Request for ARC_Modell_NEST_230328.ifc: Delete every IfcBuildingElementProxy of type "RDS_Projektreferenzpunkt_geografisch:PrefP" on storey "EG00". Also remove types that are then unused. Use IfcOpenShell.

First a look at what the model holds.

```python
import ifcopenshell
import ifcopenshell.util.element

model = ifcopenshell.open("ARC_Modell_NEST_230328.ifc")
print(model.schema)
storey = next(s for s in model.by_type("IfcBuildingStorey") if s.Name == "EG00")
proxies = [e for e in ifcopenshell.util.element.get_decomposition(storey) if e.is_a("IfcBuildingElementProxy")]
seen = {}
for e in proxies:
    element_type = ifcopenshell.util.element.get_type(e)
    name = element_type.Name if element_type not in (None, e) else None
    seen[name] = seen.get(name, 0) + 1
for name, count in sorted(seen.items(), key=str):
    print(count, "x", name)
```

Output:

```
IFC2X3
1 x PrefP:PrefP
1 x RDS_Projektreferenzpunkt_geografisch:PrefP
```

```python
import ifcopenshell
import ifcopenshell.api.root
import ifcopenshell.util.element

model = ifcopenshell.open("ARC_Modell_NEST_230328.ifc")

storey = next(s for s in model.by_type("IfcBuildingStorey") if s.Name == "EG00")
proxies = [e for e in ifcopenshell.util.element.get_decomposition(storey) if e.is_a("IfcBuildingElementProxy")]
targets = [e for e in proxies if (t := ifcopenshell.util.element.get_type(e)) not in (None, e) and t.Name == "RDS_Projektreferenzpunkt_geografisch:PrefP"]
types = {ifcopenshell.util.element.get_type(e) for e in targets} - {None, *targets}

for e in targets:
    ifcopenshell.api.root.remove_product(model, product=e)
print(len(targets), "removed")

unused = [t for t in types if not ifcopenshell.util.element.get_types(t)]
for t in unused:
    ifcopenshell.api.root.remove_product(model, product=t)
print(len(unused), "unused types removed")

model.write("ARC_Modell_NEST_230328_rev.ifc")
```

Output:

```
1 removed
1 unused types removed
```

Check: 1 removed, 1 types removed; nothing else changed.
